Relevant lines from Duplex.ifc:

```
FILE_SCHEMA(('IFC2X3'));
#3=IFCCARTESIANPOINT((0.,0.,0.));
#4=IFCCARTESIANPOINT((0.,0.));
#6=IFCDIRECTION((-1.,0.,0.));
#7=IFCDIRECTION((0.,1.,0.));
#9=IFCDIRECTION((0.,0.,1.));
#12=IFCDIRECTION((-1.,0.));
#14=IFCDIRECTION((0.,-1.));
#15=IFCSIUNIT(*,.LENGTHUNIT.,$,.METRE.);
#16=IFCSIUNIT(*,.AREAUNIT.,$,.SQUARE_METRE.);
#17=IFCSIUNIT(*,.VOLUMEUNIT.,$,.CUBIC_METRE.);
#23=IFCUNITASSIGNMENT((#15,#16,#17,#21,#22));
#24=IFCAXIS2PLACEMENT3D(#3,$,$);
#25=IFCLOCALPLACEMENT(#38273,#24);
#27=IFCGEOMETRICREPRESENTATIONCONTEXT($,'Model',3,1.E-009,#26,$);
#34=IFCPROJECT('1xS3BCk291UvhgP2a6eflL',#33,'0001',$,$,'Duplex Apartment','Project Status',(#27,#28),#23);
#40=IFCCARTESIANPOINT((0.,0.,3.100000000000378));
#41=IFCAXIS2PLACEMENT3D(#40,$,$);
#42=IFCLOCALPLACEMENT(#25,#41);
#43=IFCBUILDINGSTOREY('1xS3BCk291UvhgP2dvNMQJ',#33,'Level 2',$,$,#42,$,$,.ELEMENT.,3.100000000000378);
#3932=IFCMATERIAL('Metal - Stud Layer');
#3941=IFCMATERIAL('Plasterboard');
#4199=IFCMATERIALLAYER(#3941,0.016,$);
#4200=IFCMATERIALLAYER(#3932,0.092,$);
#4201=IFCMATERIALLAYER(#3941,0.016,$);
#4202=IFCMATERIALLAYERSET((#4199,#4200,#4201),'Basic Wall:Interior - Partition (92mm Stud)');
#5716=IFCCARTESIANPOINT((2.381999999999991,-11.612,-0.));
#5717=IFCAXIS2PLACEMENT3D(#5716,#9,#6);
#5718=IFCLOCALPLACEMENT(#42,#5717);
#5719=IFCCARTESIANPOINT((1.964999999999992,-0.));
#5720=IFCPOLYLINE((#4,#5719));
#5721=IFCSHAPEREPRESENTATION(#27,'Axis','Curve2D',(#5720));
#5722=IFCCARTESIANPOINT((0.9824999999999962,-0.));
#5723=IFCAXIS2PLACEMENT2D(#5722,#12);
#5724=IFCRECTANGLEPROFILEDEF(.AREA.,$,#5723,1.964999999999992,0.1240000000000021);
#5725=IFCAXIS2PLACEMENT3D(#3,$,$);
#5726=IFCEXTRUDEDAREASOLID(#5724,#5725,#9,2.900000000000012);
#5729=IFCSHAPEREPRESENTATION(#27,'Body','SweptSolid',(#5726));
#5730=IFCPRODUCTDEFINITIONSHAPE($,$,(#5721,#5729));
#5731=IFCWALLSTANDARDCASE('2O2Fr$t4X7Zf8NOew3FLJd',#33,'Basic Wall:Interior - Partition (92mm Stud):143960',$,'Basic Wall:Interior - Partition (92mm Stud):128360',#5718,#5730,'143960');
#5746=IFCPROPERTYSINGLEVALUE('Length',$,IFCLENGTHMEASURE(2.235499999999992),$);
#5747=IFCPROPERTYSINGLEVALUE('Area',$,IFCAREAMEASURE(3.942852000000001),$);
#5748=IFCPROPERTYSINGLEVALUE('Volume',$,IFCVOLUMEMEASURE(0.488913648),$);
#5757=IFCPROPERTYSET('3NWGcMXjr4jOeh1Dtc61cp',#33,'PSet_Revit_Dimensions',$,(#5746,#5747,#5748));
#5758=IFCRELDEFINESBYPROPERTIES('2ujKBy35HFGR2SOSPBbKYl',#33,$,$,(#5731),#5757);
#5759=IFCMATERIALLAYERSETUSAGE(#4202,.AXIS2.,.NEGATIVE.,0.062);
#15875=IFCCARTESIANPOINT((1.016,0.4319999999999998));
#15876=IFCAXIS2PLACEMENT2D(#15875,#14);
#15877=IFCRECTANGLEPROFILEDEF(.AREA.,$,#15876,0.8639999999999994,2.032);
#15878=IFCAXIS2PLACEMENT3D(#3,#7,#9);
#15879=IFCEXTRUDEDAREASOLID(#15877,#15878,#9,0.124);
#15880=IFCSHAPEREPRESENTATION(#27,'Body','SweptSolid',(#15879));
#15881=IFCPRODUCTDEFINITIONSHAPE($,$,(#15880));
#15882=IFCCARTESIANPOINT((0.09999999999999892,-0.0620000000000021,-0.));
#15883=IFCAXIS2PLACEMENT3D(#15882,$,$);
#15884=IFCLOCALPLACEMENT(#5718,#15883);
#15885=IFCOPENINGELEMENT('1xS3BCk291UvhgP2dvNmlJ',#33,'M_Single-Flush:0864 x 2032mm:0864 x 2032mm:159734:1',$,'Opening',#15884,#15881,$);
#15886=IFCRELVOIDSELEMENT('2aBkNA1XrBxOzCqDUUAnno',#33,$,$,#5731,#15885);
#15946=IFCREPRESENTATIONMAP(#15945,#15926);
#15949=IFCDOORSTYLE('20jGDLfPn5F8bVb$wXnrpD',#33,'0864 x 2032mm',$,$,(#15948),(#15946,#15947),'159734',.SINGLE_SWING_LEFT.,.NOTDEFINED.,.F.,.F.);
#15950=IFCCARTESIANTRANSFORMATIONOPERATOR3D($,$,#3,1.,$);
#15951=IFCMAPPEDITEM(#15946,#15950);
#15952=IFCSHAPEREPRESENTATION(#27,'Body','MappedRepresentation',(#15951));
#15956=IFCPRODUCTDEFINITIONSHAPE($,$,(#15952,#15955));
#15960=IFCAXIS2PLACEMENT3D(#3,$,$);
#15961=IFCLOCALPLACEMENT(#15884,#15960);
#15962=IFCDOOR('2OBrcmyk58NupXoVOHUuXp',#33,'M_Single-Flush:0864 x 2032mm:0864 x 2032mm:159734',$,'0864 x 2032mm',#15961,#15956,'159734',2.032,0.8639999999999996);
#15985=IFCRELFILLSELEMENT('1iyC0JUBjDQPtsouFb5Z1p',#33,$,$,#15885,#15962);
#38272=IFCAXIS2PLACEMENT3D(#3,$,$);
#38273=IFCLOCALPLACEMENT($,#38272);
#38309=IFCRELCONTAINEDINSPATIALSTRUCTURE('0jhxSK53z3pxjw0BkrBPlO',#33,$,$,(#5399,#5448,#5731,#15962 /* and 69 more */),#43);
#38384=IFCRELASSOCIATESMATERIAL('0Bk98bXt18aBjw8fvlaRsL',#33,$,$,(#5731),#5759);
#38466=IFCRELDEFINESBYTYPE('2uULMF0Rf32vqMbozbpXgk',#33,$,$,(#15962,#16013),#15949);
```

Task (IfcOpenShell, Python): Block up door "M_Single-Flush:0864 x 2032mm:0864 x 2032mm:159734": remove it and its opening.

```python
import ifcopenshell
import ifcopenshell.api.feature
import ifcopenshell.api.pset
import ifcopenshell.api.root
import ifcopenshell.geom
import ifcopenshell.util.element
import ifcopenshell.util.shape
import ifcopenshell.util.unit

model = ifcopenshell.open("Duplex.ifc")
area_scale = ifcopenshell.util.unit.calculate_unit_scale(model, "AREAUNIT")
volume_scale = ifcopenshell.util.unit.calculate_unit_scale(model, "VOLUMEUNIT")
settings = ifcopenshell.geom.settings()


def volume(element):
    """Net volume in cubic metres, openings subtracted."""
    shape = ifcopenshell.geom.create_shape(settings, element)
    return ifcopenshell.util.shape.get_volume(shape.geometry)


door = model.by_guid("2OBrcmyk58NupXoVOHUuXp")
opening = door.FillsVoids[0].RelatingOpeningElement
wall = opening.VoidsElements[0].RelatingBuildingElement
before = volume(wall)

ifcopenshell.api.root.remove_product(model, product=door)
ifcopenshell.api.feature.remove_feature(model, feature=opening)

after = volume(wall)
thickness = 0.124  # wall thickness in metres

# Update the wall's stored quantities.
pset = model.by_id(ifcopenshell.util.element.get_pset(wall, "PSet_Revit_Dimensions", should_inherit=False)["id"])
ifcopenshell.api.pset.edit_pset(model, pset=pset, properties={
    "Area": model.create_entity("IfcAreaMeasure", after / thickness / area_scale),
    "Volume": model.create_entity("IfcVolumeMeasure", after / volume_scale),
})

print(f"wall volume {before:.3f} -> {after:.3f} m3")

model.write("Duplex_rev.ifc")
```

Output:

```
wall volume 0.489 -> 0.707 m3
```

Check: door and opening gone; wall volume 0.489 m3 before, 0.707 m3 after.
